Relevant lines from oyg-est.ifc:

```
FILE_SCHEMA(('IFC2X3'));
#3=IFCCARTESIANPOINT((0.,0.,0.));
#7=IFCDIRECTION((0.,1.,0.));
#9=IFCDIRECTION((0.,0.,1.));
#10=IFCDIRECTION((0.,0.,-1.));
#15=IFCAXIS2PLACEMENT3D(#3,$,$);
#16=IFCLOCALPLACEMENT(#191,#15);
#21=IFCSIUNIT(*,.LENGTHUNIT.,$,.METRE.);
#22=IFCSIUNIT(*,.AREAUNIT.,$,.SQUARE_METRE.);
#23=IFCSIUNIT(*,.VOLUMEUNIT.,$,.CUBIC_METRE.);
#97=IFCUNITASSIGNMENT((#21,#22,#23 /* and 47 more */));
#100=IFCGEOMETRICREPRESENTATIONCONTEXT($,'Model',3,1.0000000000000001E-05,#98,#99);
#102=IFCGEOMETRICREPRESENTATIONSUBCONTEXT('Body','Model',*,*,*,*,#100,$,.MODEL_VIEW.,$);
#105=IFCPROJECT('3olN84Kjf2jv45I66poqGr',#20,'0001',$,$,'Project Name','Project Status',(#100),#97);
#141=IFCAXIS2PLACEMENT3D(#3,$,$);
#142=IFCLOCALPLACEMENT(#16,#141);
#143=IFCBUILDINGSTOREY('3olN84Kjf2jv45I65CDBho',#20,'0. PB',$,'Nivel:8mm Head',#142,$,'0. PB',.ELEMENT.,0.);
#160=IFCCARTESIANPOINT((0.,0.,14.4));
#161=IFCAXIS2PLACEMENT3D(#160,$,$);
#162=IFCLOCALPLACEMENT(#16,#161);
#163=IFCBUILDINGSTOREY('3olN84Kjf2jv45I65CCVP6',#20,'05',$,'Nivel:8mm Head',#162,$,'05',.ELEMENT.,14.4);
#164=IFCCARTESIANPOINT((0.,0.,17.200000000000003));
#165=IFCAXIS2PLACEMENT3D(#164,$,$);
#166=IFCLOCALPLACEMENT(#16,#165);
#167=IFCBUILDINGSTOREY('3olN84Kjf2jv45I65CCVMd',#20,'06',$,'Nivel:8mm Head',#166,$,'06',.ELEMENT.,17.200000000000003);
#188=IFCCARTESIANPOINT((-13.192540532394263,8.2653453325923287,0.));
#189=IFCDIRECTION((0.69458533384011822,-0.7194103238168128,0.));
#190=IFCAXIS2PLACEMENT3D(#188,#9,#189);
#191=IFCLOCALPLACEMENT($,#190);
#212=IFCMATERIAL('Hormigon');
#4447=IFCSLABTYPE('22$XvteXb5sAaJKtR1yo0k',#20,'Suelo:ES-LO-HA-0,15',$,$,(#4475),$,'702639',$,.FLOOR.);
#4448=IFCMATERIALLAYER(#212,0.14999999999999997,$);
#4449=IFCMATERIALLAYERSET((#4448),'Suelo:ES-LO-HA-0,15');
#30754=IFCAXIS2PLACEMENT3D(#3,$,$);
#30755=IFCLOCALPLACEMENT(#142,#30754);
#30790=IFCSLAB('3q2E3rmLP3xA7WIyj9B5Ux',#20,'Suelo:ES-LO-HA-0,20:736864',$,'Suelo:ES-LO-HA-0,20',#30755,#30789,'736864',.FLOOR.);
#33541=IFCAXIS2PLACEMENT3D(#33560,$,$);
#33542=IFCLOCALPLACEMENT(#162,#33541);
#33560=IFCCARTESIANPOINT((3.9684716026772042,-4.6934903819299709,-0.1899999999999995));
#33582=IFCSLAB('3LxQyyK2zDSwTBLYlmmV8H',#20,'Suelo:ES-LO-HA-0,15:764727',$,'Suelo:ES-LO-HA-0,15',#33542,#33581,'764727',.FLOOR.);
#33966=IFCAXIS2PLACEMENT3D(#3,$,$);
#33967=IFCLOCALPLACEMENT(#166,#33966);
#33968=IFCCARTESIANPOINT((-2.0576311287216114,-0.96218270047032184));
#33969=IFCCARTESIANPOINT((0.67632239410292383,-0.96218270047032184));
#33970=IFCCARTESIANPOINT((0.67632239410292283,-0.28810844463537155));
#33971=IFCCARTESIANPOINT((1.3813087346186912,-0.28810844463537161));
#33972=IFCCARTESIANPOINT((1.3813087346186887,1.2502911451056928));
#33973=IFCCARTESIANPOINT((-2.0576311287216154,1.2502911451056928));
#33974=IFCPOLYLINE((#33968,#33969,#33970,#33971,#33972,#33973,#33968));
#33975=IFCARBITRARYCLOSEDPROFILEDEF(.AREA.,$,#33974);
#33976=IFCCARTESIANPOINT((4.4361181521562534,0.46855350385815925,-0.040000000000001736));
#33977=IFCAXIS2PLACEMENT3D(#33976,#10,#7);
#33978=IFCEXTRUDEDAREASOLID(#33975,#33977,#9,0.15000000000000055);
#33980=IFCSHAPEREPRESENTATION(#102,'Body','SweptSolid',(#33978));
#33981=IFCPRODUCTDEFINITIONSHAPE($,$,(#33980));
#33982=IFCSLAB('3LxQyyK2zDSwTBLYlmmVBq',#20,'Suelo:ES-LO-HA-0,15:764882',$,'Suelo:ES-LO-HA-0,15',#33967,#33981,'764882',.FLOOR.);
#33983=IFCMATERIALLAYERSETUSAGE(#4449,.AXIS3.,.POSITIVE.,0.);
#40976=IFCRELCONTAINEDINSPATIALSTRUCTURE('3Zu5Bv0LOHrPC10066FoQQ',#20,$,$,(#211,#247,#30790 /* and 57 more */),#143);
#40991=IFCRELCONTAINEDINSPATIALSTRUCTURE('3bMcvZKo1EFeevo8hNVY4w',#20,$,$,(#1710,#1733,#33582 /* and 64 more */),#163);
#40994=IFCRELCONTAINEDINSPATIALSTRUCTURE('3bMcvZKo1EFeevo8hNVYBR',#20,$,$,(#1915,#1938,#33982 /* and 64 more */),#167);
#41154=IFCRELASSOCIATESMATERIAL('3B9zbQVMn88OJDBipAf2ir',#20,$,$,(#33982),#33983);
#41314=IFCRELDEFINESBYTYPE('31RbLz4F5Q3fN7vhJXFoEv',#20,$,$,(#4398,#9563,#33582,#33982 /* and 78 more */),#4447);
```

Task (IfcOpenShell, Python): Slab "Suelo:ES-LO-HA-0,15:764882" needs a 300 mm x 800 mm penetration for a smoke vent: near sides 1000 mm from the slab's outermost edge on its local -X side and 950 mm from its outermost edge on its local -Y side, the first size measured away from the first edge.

```python
import numpy as np
import ifcopenshell
import ifcopenshell.api.feature
import ifcopenshell.api.geometry
import ifcopenshell.api.root
import ifcopenshell.geom
import ifcopenshell.util.placement
import ifcopenshell.util.representation
import ifcopenshell.util.shape
import ifcopenshell.util.unit

model = ifcopenshell.open("oyg-est.ifc")
unit_scale = ifcopenshell.util.unit.calculate_unit_scale(model)
settings = ifcopenshell.geom.settings()


def volume(element):
    """Net volume in cubic metres, openings subtracted."""
    shape = ifcopenshell.geom.create_shape(settings, element)
    return ifcopenshell.util.shape.get_volume(shape.geometry)


slab = model.by_guid("3LxQyyK2zDSwTBLYlmmVBq")
before = volume(slab)

# Extent in the slab's own axes, in metres. The edges named are its -X and -Y sides.
slab_shape = ifcopenshell.geom.create_shape(settings, slab)
vertices = ifcopenshell.util.shape.get_vertices(slab_shape.geometry)
x_min, y_min, bottom = vertices.min(axis=0)
top = vertices[:, 2].max()

opening = ifcopenshell.api.root.create_entity(model, ifc_class="IfcOpeningElement", name="Smoke vent opening")
context = ifcopenshell.util.representation.get_context(model, "Model", "Body", "MODEL_VIEW")
width, depth = 0.3, 0.8
outline = [(0.0, 0.0), (width, 0.0), (width, depth), (0.0, depth), (0.0, 0.0)]
# Overshoot both faces by 50 mm so the cut is clean.
shape = ifcopenshell.api.geometry.add_slab_representation(
    model, context=context, depth=top - bottom + 0.1, polyline=outline
)
ifcopenshell.api.geometry.assign_representation(model, product=opening, representation=shape)

matrix = ifcopenshell.util.placement.get_local_placement(slab.ObjectPlacement)
matrix[:, 3] = matrix @ np.append(np.array([x_min + 1, y_min + 0.95, bottom - 0.05]) / unit_scale, 1.0)
ifcopenshell.api.geometry.edit_object_placement(model, product=opening, matrix=matrix, is_si=False)
ifcopenshell.api.feature.add_feature(model, feature=opening, element=slab)

after = volume(slab)

print(f"slab volume {before:.3f} -> {after:.3f} m3")

model.write("oyg-est_updated.ifc")
```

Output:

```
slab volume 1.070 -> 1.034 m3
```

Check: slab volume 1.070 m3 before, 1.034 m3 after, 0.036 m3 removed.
